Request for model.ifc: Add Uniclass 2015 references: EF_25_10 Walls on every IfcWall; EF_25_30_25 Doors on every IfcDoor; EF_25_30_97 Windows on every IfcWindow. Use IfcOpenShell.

First a look at what the model holds.

```python
import ifcopenshell

model = ifcopenshell.open("model.ifc")
print(model.schema)
print("classifications:", [c.Name for c in model.by_type("IfcClassification")])
for ifc_class in ("IfcDoor", "IfcRoof", "IfcStair", "IfcWall", "IfcWindow"):
    print(ifc_class, len(model.by_type(ifc_class)))
```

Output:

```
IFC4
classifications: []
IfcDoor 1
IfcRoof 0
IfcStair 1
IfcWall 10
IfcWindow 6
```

```python
import ifcopenshell
import ifcopenshell.api.classification

model = ifcopenshell.open("model.ifc")

system = ifcopenshell.api.classification.add_classification(model, classification="Uniclass 2015")

codes = {
    "IfcWall": ("EF_25_10", "Walls"),
    "IfcDoor": ("EF_25_30_25", "Doors"),
    "IfcWindow": ("EF_25_30_97", "Windows"),
}
for ifc_class, (code, name) in codes.items():
    products = model.by_type(ifc_class)
    ifcopenshell.api.classification.add_reference(
        model, products=products, classification=system, identification=code, name=name
    )
    print(code, len(products))

model.write("model_rev.ifc")
```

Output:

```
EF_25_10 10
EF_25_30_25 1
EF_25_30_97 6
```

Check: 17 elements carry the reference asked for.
